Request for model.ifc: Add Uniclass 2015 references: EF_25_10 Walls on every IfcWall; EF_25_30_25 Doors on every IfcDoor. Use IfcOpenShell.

First a look at what the model holds.

```python
import ifcopenshell

model = ifcopenshell.open("model.ifc")
print(model.schema)
print("classifications:", [c.Name for c in model.by_type("IfcClassification")])
for ifc_class in ("IfcDoor", "IfcRoof", "IfcStair", "IfcWall", "IfcWindow"):
    print(ifc_class, len(model.by_type(ifc_class)))
```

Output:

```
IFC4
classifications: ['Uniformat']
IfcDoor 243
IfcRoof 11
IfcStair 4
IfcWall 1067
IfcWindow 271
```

```python
import ifcopenshell
import ifcopenshell.api.classification

model = ifcopenshell.open("model.ifc")

system = ifcopenshell.api.classification.add_classification(model, classification="Uniclass 2015")

codes = {
    "IfcWall": ("EF_25_10", "Walls"),
    "IfcDoor": ("EF_25_30_25", "Doors"),
}
for ifc_class, (code, name) in codes.items():
    products = model.by_type(ifc_class)
    ifcopenshell.api.classification.add_reference(
        model, products=products, classification=system, identification=code, name=name
    )
    print(code, len(products))

model.write("model-out.ifc")
```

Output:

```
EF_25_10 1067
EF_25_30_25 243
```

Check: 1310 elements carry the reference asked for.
